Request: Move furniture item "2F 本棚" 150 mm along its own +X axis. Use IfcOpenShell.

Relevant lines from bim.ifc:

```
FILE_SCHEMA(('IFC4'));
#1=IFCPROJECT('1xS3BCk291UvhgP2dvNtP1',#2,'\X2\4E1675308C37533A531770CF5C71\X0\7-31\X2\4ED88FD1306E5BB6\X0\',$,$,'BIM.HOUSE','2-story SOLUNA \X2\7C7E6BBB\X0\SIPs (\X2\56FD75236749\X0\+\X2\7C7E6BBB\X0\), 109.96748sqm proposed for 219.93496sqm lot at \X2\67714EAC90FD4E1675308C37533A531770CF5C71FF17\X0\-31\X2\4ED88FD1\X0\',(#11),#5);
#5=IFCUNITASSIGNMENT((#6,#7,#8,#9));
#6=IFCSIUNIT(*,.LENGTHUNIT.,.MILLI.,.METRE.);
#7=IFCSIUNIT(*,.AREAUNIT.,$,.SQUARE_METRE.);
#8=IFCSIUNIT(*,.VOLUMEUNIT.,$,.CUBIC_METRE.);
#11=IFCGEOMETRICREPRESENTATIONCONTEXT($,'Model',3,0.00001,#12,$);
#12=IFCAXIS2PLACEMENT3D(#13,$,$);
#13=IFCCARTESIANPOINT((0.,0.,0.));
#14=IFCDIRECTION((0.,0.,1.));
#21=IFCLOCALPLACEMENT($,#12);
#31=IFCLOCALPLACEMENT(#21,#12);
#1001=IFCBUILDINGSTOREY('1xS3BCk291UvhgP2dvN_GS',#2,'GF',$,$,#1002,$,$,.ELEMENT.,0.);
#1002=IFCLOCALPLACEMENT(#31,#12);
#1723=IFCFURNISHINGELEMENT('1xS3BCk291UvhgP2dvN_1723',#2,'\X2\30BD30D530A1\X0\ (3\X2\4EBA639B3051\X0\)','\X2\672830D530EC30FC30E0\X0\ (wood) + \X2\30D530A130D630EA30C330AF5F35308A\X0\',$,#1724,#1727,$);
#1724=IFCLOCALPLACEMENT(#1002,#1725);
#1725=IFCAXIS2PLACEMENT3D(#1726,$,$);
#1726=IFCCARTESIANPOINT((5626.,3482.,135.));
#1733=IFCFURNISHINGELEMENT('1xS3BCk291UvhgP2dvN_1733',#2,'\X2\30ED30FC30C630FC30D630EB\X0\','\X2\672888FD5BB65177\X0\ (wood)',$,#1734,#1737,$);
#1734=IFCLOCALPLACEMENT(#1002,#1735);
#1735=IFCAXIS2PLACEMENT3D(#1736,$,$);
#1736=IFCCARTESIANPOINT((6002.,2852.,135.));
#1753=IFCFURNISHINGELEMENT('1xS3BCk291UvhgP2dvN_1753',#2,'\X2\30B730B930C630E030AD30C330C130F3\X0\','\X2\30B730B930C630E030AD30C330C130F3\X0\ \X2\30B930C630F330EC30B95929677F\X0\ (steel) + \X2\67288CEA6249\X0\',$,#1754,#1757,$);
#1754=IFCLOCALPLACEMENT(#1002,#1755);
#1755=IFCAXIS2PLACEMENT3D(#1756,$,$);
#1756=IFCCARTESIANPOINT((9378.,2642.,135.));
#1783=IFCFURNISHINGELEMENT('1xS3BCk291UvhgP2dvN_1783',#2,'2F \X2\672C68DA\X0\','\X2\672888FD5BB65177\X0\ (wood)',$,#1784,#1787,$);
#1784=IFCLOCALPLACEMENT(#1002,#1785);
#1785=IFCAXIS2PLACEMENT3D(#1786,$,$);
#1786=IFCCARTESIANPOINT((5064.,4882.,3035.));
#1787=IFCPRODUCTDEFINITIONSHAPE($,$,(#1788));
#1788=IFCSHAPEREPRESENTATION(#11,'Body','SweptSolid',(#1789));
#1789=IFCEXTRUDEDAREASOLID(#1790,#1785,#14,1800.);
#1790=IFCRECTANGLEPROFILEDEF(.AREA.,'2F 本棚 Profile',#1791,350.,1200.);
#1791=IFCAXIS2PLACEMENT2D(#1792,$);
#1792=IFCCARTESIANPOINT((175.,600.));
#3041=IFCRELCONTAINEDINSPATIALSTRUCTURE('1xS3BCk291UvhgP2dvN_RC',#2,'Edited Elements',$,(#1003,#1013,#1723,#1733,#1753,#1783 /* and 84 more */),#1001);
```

```python
import ifcopenshell
import ifcopenshell.api.geometry
import ifcopenshell.util.placement

model = ifcopenshell.open("bim.ifc")

item = model.by_guid("1xS3BCk291UvhgP2dvN_1783")
matrix = ifcopenshell.util.placement.get_local_placement(item.ObjectPlacement)
matrix[:3, 3] += matrix[:3, 0] * 150.0
ifcopenshell.api.geometry.edit_object_placement(model, product=item, matrix=matrix, is_si=False)

print(ifcopenshell.util.placement.get_local_placement(item.ObjectPlacement).round(3) + 0.0)

model.write("bim_v2.ifc")
```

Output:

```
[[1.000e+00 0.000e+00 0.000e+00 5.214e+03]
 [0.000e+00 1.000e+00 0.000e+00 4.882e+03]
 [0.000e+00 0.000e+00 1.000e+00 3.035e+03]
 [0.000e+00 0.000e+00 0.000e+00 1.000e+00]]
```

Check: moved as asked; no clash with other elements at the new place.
